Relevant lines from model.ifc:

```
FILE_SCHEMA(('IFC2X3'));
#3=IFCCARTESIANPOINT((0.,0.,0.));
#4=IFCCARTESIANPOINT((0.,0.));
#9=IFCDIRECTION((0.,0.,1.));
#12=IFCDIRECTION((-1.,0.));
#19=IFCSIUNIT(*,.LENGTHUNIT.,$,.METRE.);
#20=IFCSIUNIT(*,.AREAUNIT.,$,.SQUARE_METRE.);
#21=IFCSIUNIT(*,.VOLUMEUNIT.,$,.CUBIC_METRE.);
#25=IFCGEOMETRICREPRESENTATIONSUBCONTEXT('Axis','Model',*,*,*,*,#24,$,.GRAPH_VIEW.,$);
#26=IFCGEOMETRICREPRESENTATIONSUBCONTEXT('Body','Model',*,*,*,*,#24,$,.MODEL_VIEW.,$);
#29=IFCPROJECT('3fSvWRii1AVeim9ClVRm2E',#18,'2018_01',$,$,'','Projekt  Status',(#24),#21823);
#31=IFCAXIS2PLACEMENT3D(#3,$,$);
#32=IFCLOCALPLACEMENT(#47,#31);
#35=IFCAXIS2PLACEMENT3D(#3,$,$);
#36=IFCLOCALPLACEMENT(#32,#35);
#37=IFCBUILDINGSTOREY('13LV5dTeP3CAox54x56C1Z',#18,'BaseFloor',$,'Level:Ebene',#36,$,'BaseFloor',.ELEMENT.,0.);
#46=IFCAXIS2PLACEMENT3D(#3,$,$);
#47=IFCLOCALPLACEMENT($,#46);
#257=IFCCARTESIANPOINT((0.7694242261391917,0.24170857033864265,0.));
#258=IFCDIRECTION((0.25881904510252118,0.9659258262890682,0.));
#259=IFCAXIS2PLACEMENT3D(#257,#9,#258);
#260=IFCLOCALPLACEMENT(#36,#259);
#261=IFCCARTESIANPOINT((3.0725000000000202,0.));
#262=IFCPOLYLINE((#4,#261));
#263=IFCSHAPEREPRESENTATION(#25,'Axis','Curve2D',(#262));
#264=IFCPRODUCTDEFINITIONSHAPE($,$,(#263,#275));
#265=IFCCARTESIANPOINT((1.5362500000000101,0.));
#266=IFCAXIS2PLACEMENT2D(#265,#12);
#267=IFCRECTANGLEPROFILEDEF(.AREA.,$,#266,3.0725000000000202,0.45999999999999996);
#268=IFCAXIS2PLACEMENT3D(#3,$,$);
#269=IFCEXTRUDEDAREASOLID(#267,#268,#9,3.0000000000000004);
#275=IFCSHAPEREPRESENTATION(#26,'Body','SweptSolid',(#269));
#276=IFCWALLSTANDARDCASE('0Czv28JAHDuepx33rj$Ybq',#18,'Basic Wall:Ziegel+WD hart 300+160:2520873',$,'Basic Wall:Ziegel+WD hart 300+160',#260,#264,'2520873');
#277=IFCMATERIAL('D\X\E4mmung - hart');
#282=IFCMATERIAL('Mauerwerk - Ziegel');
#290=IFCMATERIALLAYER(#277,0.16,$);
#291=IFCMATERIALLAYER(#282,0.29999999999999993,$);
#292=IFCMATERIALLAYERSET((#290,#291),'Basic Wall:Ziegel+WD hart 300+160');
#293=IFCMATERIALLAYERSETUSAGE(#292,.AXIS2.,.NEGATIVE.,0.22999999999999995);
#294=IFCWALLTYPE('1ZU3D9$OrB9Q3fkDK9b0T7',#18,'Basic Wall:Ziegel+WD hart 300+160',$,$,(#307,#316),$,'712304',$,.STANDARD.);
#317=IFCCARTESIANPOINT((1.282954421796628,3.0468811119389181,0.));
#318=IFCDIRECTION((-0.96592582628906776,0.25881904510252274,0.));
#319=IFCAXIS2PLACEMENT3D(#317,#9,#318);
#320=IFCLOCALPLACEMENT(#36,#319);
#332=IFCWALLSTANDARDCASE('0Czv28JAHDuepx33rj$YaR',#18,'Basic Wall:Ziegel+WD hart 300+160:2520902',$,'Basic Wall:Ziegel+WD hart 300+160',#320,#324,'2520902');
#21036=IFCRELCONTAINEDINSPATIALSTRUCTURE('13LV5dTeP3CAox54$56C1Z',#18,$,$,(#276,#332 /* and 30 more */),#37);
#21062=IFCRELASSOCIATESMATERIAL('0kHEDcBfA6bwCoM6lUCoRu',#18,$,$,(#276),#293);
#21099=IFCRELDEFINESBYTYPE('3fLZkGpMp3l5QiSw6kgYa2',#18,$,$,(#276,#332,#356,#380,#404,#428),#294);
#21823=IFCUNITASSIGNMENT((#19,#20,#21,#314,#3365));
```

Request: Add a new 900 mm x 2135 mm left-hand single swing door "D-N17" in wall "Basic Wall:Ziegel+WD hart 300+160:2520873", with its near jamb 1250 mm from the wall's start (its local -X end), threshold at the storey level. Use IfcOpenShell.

```python
import numpy as np
import ifcopenshell
import ifcopenshell.api.feature
import ifcopenshell.api.geometry
import ifcopenshell.api.root
import ifcopenshell.api.spatial
import ifcopenshell.api.type
import ifcopenshell.geom
import ifcopenshell.util.element
import ifcopenshell.util.placement
import ifcopenshell.util.representation
import ifcopenshell.util.shape
import ifcopenshell.util.unit

model = ifcopenshell.open("model.ifc")
unit_scale = ifcopenshell.util.unit.calculate_unit_scale(model)
settings = ifcopenshell.geom.settings()


def volume(element):
    """Net volume in cubic metres, openings subtracted."""
    shape = ifcopenshell.geom.create_shape(settings, element)
    return ifcopenshell.util.shape.get_volume(shape.geometry)


wall = model.by_guid("0Czv28JAHDuepx33rj$Ybq")
storey = ifcopenshell.util.element.get_container(wall, ifc_class="IfcBuildingStorey")
context = ifcopenshell.util.representation.get_context(model, "Model", "Body", "MODEL_VIEW")
before = volume(wall)

width, height, from_end, sill = 0.9, 2.135, 1.25, 0.0  # metres

# The wall runs along its own X axis, and the end named is its -X end.
wall_shape = ifcopenshell.geom.create_shape(settings, wall)
x, y, z = ifcopenshell.util.shape.get_vertices(wall_shape.geometry).T
start = x.min() + from_end
face, thickness = float(y.min()), float(y.max() - y.min())
wall_matrix = ifcopenshell.util.placement.get_local_placement(wall.ObjectPlacement)
level = ifcopenshell.util.placement.get_local_placement(storey.ObjectPlacement)[2, 3]


def in_wall(x, y):
    """Placement at x, y metres in the wall's axes, at sill height."""
    matrix = wall_matrix.copy()
    matrix[:, 3] = wall_matrix @ np.array([x / unit_scale, y / unit_scale, 0.0, 1.0])
    matrix[2, 3] = level + sill / unit_scale
    return matrix


# Opening: a box that overshoots both wall faces by 50 mm.
opening = ifcopenshell.api.root.create_entity(model, ifc_class="IfcOpeningElement")
box = ifcopenshell.api.geometry.add_wall_representation(
    model, context=context, length=width, height=height, thickness=thickness + 0.1
)
ifcopenshell.api.geometry.assign_representation(model, product=opening, representation=box)
ifcopenshell.api.geometry.edit_object_placement(model, product=opening, matrix=in_wall(start, face - 0.05), is_si=False)
ifcopenshell.api.feature.add_feature(model, feature=opening, element=wall)

door = ifcopenshell.api.root.create_entity(model, ifc_class="IfcDoor", name="D-N17")
door.OverallWidth, door.OverallHeight = width / unit_scale, height / unit_scale
body = ifcopenshell.api.geometry.add_door_representation(
    model,
    context=context,
    overall_width=door.OverallWidth,
    overall_height=door.OverallHeight,
    operation_type="SINGLE_SWING_LEFT",
    lining_properties={"LiningDepth": thickness / unit_scale, "ThresholdDepth": thickness / unit_scale},
)
ifcopenshell.api.geometry.assign_representation(model, product=door, representation=body)
ifcopenshell.api.spatial.assign_container(model, products=[door], relating_structure=storey)
fills = ifcopenshell.api.feature.add_filling(model, opening=opening, element=door)
fills.OwnerHistory = door.OwnerHistory  # required in IFC2X3

# IFC2X3 keeps the operation on the door style.
style = ifcopenshell.api.root.create_entity(model, ifc_class="IfcDoorStyle", name="D-N17")
style.OperationType, style.ConstructionType = "SINGLE_SWING_LEFT", "NOTDEFINED"
style.ParameterTakesPrecedence = style.Sizeable = False
ifcopenshell.api.type.assign_type(model, related_objects=[door], relating_type=style)

# The lining spans the wall, so the door starts at the wall face.
ifcopenshell.api.geometry.edit_object_placement(model, product=door, matrix=in_wall(start, face), is_si=False)

after = volume(wall)

print(f"wall volume {before:.3f} -> {after:.3f} m3")

model.write("model_rev.ifc")
```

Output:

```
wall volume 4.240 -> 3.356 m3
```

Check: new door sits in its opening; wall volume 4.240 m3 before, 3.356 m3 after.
